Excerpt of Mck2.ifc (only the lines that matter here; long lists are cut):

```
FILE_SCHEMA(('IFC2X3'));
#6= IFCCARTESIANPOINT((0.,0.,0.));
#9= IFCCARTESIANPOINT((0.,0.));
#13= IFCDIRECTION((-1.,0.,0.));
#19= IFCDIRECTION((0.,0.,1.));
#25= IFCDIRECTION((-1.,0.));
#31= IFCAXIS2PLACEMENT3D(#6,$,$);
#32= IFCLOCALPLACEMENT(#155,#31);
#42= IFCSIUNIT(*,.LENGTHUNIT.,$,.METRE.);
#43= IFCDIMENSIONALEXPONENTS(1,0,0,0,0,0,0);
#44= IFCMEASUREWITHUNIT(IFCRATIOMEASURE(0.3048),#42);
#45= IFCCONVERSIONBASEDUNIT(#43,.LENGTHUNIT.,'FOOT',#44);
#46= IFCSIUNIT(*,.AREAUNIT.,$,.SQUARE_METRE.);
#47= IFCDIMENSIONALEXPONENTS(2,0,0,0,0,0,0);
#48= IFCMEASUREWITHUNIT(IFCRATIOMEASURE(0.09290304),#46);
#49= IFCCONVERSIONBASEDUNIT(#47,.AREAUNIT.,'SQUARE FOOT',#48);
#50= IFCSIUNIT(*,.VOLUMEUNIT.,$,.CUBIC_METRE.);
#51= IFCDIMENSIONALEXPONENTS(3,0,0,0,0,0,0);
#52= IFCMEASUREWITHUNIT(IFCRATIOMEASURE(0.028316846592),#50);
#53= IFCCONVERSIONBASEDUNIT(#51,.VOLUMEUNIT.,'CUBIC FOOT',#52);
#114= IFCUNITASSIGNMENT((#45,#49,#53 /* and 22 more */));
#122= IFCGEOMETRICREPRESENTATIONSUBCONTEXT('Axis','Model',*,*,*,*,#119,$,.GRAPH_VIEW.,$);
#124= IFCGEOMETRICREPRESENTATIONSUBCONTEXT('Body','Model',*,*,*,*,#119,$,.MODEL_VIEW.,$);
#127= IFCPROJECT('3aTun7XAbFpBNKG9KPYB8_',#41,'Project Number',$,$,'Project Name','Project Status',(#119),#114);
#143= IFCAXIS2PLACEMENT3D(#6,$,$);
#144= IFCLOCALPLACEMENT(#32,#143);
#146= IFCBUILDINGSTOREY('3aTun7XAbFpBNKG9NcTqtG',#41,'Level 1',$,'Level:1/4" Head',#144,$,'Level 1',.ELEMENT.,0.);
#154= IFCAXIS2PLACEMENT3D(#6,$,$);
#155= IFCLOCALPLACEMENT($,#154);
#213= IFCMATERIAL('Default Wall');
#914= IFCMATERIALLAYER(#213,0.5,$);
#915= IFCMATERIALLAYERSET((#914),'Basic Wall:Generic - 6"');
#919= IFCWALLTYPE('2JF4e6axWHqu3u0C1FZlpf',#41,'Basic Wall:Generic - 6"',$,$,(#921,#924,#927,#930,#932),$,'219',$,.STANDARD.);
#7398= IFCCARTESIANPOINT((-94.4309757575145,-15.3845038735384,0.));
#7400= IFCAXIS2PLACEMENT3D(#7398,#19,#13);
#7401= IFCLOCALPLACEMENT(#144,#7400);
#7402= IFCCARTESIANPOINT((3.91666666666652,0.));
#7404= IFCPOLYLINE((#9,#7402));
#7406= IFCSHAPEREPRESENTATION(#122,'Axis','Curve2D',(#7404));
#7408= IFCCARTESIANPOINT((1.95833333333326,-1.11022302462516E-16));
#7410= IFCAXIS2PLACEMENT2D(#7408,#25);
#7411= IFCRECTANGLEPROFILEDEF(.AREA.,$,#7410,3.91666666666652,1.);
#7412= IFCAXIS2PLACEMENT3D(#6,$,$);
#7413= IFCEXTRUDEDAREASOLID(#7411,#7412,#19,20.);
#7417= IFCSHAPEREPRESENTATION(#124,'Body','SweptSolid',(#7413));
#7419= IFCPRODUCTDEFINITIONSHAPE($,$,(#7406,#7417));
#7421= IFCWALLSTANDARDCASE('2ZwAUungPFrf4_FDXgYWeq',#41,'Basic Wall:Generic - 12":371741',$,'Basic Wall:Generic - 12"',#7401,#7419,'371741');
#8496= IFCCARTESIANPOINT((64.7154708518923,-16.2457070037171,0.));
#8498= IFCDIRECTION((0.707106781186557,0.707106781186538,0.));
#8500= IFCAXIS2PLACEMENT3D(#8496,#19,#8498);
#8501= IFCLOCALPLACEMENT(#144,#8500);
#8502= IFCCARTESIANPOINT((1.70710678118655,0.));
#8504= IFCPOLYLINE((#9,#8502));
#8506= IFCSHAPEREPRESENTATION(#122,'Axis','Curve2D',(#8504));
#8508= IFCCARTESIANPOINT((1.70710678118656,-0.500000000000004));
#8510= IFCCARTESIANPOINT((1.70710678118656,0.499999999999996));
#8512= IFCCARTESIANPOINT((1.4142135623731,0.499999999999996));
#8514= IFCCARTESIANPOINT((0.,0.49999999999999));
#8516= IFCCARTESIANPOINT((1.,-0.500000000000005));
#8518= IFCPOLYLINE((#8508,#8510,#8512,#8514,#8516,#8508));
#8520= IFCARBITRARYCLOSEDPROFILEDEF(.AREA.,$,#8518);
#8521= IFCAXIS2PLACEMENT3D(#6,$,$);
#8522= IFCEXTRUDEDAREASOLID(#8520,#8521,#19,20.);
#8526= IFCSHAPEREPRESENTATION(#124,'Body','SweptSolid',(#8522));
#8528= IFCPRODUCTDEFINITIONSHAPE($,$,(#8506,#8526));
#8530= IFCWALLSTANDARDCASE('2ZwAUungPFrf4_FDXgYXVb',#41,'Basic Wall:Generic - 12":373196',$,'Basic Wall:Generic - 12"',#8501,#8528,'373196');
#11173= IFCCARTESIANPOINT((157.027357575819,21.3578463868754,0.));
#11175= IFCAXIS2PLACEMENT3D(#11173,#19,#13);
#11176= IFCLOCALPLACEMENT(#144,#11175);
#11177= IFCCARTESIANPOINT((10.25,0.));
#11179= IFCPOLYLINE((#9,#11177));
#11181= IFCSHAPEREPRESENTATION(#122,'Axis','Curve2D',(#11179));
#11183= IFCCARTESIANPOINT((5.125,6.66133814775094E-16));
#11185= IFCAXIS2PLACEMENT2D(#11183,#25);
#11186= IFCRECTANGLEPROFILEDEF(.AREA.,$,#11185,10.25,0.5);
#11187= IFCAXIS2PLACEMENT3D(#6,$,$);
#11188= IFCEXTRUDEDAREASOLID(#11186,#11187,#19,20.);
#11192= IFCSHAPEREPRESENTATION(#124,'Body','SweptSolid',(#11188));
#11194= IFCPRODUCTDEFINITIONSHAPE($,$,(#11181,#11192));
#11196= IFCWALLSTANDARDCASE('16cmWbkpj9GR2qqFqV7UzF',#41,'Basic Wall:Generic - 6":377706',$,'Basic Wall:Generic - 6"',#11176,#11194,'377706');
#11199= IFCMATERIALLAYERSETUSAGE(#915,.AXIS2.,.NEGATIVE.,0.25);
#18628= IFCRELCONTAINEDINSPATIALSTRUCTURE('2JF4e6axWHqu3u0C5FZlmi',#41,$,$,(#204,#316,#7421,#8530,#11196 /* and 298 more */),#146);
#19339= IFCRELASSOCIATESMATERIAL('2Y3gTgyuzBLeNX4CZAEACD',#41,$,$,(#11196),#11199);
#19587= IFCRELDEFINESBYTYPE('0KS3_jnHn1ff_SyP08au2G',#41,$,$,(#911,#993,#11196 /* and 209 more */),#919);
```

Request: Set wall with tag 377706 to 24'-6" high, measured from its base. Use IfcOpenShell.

```python
import ifcopenshell
import ifcopenshell.geom
import ifcopenshell.util.representation
import ifcopenshell.util.shape
import ifcopenshell.util.unit

model = ifcopenshell.open("Mck2.ifc")
unit_scale = ifcopenshell.util.unit.calculate_unit_scale(model)
settings = ifcopenshell.geom.settings()


def volume(element):
    """Net volume in cubic metres, openings subtracted."""
    shape = ifcopenshell.geom.create_shape(settings, element)
    return ifcopenshell.util.shape.get_volume(shape.geometry)


wall = model.by_id(11196)
before = volume(wall)

body = ifcopenshell.util.representation.get_representation(wall, "Model", "Body")
solid = body.Items[0]
old_height = solid.Depth
solid.Depth = 294 * 0.0254 / unit_scale
after = volume(wall)

print(f"height {old_height:g} -> {solid.Depth:g}, volume {before:.3f} -> {after:.3f} m3")

model.write("Mck2_edited.ifc")
```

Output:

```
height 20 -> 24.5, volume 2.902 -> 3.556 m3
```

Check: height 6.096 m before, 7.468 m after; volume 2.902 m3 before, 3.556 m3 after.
